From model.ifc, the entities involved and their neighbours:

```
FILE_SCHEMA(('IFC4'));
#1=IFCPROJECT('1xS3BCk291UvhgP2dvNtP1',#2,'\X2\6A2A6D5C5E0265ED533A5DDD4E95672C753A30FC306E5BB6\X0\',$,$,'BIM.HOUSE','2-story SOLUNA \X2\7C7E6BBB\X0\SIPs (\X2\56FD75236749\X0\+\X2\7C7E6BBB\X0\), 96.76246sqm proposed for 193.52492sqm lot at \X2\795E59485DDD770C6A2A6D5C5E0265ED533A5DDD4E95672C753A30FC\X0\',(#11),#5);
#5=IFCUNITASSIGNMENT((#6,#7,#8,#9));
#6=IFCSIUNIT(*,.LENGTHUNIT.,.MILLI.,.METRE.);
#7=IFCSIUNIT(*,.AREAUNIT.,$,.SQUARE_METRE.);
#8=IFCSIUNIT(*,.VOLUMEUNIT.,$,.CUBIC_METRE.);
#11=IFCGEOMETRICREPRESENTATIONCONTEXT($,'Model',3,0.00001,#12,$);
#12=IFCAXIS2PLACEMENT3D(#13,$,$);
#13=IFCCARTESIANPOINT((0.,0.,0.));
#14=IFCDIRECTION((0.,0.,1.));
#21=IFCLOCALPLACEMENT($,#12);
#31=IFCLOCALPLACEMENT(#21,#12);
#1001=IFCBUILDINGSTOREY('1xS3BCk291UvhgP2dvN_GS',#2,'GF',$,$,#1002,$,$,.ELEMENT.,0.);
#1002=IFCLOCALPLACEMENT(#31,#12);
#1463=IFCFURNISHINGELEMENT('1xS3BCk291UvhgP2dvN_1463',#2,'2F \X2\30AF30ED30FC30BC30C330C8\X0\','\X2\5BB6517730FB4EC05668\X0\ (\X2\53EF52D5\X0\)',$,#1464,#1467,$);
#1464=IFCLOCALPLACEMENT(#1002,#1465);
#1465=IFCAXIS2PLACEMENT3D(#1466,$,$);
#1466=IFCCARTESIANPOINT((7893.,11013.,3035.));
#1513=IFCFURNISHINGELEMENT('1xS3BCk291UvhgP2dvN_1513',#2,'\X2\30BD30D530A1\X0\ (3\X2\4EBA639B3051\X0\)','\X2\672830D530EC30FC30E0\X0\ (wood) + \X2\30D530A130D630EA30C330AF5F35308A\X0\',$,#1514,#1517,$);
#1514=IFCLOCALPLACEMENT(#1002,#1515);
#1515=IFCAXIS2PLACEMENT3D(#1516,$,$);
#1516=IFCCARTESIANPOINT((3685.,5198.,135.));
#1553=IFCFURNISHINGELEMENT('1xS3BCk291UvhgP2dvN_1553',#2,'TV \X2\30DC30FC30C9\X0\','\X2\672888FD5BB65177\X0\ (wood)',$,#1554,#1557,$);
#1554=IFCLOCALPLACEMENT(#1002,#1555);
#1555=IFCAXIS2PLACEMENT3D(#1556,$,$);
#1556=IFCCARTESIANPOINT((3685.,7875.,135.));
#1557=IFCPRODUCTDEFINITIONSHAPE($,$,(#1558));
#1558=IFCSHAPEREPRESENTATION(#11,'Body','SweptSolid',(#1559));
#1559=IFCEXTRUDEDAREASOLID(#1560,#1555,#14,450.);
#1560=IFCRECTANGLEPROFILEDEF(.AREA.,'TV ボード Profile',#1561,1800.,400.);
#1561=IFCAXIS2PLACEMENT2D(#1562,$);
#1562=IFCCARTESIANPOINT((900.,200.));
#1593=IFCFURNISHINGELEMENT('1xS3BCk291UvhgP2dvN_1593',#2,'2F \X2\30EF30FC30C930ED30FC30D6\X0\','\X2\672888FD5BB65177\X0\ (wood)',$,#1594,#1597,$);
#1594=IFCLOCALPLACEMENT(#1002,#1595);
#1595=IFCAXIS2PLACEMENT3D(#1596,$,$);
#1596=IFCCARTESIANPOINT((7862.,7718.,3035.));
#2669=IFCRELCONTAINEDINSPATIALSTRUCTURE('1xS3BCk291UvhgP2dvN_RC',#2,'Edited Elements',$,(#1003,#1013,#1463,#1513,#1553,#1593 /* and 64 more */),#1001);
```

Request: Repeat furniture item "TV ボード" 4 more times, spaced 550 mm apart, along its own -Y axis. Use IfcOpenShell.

```python
import ifcopenshell
import ifcopenshell.api.geometry
import ifcopenshell.api.root
import ifcopenshell.util.element
import ifcopenshell.util.placement
import ifcopenshell.util.unit

model = ifcopenshell.open("model.ifc")
unit_scale = ifcopenshell.util.unit.calculate_unit_scale(model)


def reuse_history(source, copy):
    """copy_class also copies each property set's owner history, people and application; keep the originals."""
    for rel in copy.IsDefinedBy:
        if rel.is_a("IfcRelDefinesByProperties") and (history := rel.RelatingPropertyDefinition.OwnerHistory):
            rel.RelatingPropertyDefinition.OwnerHistory = source.OwnerHistory
            ifcopenshell.util.element.remove_deep2(model, history)


source = model.by_guid("1xS3BCk291UvhgP2dvN_1553")
base = ifcopenshell.util.placement.get_local_placement(source.ObjectPlacement)
step = -base[:3, 1] * 0.55 / unit_scale

for i in range(1, 5):
    copy = ifcopenshell.api.root.copy_class(model, product=source)
    copy.Representation = ifcopenshell.util.element.copy_deep(
        model, source.Representation, exclude=["IfcGeometricRepresentationContext", "IfcRepresentationMap"]
    )
    reuse_history(source, copy)
    matrix = base.copy()
    matrix[:3, 3] += i * step
    print("added at", matrix[:3, 3].round(3) + 0.0)
    ifcopenshell.api.geometry.edit_object_placement(model, product=copy, matrix=matrix, is_si=False)

model.write("model_updated.ifc")
```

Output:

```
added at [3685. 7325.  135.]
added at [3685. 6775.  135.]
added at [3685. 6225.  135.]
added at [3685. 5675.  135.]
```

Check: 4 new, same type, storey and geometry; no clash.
